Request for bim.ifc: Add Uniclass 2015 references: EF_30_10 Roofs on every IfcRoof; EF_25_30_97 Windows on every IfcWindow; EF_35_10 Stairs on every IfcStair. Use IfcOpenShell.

First a look at what the model holds.

```python
import ifcopenshell

model = ifcopenshell.open("bim.ifc")
print(model.schema)
print("classifications:", [c.Name for c in model.by_type("IfcClassification")])
for ifc_class in ("IfcDoor", "IfcRoof", "IfcStair", "IfcWall", "IfcWindow"):
    print(ifc_class, len(model.by_type(ifc_class)))
```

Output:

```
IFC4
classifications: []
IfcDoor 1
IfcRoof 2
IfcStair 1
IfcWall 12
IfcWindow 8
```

```python
import ifcopenshell
import ifcopenshell.api.classification

model = ifcopenshell.open("bim.ifc")

system = ifcopenshell.api.classification.add_classification(model, classification="Uniclass 2015")

codes = {
    "IfcRoof": ("EF_30_10", "Roofs"),
    "IfcWindow": ("EF_25_30_97", "Windows"),
    "IfcStair": ("EF_35_10", "Stairs"),
}
for ifc_class, (code, name) in codes.items():
    products = model.by_type(ifc_class)
    ifcopenshell.api.classification.add_reference(
        model, products=products, classification=system, identification=code, name=name
    )
    print(code, len(products))

model.write("bim_rev.ifc")
```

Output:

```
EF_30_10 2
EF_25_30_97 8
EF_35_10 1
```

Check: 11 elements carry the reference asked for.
